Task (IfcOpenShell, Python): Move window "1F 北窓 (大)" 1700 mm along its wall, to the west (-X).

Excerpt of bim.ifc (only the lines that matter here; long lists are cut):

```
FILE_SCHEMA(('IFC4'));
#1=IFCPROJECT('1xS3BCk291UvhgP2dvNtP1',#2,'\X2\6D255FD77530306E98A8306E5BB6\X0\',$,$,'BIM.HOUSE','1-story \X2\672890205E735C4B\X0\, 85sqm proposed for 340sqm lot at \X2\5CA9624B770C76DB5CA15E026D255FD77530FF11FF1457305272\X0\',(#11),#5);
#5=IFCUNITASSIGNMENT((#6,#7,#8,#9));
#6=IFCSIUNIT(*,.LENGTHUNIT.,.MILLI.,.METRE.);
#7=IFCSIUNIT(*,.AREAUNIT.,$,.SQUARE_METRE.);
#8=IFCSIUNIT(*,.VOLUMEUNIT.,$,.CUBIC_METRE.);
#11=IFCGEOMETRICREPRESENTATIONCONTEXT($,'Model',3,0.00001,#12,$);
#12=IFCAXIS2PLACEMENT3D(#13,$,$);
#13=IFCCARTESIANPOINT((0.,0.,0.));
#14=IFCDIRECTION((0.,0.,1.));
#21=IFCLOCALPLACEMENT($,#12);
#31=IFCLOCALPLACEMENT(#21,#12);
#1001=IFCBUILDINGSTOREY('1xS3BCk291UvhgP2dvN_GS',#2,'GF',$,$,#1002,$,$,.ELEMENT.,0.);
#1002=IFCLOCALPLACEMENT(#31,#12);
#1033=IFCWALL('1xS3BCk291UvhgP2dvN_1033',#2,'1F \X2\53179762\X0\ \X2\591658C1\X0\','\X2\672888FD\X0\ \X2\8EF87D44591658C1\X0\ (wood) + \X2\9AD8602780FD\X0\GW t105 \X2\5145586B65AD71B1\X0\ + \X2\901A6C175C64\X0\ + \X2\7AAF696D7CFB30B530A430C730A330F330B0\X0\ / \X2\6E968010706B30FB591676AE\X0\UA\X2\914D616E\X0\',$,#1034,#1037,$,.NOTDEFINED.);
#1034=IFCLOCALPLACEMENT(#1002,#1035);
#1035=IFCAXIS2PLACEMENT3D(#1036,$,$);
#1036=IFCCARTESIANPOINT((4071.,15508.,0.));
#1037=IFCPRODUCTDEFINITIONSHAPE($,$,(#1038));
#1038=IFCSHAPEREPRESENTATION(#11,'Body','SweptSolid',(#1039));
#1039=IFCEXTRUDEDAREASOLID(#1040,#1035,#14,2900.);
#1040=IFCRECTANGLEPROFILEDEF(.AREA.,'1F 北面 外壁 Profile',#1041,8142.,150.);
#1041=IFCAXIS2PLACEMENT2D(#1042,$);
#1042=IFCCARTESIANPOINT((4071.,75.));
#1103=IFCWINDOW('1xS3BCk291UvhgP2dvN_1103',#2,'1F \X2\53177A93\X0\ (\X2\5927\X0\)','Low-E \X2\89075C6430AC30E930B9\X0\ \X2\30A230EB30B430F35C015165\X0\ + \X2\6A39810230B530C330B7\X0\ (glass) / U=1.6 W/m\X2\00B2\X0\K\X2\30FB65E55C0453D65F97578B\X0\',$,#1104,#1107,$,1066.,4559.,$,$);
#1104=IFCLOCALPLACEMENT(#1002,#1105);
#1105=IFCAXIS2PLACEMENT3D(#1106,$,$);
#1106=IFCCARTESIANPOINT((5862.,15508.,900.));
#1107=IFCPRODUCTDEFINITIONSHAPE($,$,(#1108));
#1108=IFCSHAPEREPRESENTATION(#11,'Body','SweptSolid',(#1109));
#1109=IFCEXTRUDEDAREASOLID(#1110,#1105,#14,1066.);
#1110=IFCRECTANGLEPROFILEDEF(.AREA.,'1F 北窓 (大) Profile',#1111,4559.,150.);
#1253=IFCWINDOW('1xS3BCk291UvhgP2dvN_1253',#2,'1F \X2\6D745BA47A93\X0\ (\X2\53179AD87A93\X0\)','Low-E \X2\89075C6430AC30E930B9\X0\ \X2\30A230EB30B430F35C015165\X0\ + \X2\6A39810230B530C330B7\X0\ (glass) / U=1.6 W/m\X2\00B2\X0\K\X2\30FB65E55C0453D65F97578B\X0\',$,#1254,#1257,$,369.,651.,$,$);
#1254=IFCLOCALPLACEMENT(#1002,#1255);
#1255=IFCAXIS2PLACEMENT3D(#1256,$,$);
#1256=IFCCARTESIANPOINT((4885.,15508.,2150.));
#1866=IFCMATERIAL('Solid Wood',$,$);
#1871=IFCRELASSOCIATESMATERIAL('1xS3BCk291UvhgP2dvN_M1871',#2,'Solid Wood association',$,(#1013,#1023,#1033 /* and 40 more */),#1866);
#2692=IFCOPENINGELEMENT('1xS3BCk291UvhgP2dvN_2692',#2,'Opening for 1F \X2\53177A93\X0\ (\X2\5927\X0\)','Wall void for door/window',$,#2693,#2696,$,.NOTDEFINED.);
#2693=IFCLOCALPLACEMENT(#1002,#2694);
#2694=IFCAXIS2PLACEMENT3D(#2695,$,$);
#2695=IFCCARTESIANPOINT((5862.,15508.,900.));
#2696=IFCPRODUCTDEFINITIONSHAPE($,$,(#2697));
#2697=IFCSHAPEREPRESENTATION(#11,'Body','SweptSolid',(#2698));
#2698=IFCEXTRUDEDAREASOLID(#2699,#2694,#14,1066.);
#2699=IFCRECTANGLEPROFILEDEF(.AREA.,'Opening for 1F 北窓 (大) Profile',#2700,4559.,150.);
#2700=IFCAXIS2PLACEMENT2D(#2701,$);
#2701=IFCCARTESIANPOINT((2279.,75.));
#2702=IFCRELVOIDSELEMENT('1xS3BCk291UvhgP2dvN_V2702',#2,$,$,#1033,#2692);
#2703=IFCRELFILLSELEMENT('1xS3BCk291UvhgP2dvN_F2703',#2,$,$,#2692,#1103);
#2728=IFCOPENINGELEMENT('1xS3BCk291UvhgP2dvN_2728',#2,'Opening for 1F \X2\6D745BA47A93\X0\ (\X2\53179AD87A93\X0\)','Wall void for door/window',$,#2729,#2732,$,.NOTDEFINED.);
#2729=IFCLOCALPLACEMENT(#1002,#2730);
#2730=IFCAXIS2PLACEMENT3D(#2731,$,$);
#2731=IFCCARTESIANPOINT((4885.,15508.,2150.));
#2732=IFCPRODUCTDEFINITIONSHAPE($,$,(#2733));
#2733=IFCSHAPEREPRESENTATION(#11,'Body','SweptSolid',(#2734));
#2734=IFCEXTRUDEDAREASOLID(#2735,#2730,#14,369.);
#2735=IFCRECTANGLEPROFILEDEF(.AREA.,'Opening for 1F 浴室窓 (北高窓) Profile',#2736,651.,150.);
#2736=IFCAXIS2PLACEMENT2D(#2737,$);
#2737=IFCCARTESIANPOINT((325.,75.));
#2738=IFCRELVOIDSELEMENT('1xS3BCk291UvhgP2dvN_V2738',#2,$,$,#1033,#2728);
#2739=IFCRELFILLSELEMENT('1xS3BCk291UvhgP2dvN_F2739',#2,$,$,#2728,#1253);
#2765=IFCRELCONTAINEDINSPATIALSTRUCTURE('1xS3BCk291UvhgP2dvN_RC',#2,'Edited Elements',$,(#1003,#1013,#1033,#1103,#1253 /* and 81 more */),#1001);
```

```python
import ifcopenshell
import ifcopenshell.api.geometry
import ifcopenshell.util.placement
import ifcopenshell.util.unit

model = ifcopenshell.open("bim.ifc")
unit_scale = ifcopenshell.util.unit.calculate_unit_scale(model)

window = model.by_id(1103)
opening = window.FillsVoids[0].RelatingOpeningElement
wall = opening.VoidsElements[0].RelatingBuildingElement

wall_matrix = ifcopenshell.util.placement.get_local_placement(wall.ObjectPlacement)
shift = wall_matrix[:3, 0] * -1.7 / unit_scale
before = ifcopenshell.util.placement.get_local_placement(window.ObjectPlacement)[:3, 3].copy()

# The window is not placed relative to its opening, so move both.
for product in (opening, window):
    matrix = ifcopenshell.util.placement.get_local_placement(product.ObjectPlacement)
    matrix[:3, 3] += shift
    ifcopenshell.api.geometry.edit_object_placement(model, product=product, matrix=matrix, is_si=False)

after = ifcopenshell.util.placement.get_local_placement(window.ObjectPlacement)[:3, 3]
print("window moved by", (after - before).round(3) + 0.0)

model.write("bim_edited.ifc")
```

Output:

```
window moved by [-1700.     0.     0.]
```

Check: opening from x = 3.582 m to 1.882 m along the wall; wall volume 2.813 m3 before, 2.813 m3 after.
